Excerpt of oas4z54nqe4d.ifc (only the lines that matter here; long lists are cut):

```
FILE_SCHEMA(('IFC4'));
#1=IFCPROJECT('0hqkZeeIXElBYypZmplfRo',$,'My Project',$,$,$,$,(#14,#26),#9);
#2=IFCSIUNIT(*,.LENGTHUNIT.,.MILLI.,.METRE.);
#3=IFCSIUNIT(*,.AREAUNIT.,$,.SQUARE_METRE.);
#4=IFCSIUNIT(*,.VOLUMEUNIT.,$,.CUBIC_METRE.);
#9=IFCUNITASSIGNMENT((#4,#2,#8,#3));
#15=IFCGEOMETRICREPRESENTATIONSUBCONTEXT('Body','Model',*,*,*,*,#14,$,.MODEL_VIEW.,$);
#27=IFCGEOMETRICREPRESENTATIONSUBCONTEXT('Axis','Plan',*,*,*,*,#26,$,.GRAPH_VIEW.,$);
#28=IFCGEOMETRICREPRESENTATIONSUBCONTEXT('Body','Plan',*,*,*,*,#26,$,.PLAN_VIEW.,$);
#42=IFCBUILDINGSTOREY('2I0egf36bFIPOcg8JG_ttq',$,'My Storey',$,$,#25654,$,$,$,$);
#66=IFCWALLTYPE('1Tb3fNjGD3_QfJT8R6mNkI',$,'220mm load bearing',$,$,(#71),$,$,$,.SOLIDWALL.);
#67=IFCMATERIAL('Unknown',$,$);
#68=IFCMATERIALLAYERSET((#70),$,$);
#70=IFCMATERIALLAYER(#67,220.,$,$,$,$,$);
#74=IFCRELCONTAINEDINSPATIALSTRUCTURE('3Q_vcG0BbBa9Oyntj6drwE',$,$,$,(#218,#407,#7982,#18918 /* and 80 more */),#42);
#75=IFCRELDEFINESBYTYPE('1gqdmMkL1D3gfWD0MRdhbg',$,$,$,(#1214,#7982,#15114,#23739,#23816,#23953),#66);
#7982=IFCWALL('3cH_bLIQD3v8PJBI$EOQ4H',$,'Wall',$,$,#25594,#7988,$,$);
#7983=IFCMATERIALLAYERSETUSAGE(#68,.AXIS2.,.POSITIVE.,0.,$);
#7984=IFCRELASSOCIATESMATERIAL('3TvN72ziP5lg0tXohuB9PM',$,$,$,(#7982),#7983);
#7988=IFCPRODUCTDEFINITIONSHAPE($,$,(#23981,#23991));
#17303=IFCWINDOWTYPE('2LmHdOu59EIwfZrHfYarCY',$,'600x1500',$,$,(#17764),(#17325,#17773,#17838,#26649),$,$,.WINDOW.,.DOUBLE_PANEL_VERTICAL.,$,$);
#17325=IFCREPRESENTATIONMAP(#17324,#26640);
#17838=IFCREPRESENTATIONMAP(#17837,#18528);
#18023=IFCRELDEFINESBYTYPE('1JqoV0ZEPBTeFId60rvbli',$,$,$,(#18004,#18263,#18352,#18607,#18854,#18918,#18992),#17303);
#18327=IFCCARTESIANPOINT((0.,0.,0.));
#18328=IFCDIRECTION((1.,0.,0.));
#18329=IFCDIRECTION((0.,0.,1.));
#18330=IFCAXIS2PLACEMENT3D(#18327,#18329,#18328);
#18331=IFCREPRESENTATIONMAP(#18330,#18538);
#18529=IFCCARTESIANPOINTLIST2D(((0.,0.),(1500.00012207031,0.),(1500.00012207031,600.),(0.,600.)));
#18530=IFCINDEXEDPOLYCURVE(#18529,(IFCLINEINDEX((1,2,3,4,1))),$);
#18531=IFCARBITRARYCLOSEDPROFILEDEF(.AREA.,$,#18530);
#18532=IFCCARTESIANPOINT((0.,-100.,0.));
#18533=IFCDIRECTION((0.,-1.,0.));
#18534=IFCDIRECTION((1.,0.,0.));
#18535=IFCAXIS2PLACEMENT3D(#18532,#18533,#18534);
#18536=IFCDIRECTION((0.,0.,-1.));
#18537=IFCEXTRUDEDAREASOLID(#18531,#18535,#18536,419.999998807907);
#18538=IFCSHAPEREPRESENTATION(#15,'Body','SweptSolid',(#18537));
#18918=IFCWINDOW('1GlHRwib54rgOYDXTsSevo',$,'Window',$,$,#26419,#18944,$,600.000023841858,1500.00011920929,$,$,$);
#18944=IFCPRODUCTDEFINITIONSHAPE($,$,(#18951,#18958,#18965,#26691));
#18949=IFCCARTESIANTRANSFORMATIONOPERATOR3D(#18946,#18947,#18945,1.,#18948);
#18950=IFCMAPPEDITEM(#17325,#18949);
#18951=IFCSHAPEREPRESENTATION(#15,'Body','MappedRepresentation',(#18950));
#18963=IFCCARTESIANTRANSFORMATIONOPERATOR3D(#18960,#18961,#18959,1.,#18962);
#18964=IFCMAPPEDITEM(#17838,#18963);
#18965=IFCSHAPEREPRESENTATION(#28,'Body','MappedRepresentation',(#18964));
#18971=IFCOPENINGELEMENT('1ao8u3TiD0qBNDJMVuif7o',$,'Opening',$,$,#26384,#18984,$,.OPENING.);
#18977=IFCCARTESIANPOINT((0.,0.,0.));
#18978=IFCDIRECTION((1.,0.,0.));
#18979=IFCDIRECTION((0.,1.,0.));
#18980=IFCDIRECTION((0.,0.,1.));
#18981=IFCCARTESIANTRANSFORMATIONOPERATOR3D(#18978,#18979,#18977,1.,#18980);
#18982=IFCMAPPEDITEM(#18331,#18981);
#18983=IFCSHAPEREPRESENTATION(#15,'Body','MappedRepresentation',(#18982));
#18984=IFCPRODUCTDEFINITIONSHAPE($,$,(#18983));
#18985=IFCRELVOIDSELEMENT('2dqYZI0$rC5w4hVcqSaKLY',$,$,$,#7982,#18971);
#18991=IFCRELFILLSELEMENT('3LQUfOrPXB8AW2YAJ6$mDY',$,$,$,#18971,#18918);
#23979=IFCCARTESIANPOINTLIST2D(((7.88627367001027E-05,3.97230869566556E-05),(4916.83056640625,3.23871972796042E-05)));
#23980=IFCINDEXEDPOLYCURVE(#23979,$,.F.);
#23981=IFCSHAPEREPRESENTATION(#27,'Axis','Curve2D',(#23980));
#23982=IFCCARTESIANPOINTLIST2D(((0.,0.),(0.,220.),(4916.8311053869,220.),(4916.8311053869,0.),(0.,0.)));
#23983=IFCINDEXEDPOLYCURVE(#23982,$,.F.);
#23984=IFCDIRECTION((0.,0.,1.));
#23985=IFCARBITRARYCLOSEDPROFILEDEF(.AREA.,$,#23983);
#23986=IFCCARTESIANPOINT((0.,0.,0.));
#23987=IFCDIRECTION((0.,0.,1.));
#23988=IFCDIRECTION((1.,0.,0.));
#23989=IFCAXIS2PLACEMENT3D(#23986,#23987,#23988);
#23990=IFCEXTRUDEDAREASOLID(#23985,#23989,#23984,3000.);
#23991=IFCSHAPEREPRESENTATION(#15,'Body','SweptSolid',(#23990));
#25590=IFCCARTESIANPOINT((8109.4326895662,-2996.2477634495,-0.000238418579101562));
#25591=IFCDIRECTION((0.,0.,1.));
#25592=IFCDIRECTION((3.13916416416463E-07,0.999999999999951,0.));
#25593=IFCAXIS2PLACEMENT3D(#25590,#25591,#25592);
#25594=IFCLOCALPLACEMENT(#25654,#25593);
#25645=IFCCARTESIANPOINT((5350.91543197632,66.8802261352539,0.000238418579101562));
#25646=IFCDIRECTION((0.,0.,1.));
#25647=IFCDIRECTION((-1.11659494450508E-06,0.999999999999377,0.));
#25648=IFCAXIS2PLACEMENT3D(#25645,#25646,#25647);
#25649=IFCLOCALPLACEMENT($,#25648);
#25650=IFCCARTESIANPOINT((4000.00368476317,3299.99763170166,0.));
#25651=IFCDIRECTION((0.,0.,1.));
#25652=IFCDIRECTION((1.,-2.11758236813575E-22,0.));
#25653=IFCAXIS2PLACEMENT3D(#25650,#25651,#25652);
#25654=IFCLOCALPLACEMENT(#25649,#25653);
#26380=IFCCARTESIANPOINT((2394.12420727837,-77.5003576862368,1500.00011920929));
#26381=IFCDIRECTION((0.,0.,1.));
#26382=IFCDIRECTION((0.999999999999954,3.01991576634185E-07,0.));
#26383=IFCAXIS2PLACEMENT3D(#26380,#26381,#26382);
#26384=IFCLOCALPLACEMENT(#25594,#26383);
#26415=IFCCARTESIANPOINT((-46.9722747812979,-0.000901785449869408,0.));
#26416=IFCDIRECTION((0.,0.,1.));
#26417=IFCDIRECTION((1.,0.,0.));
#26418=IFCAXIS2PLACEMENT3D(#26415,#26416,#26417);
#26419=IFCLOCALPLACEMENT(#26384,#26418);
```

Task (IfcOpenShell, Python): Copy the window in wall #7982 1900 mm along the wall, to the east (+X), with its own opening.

```python
import ifcopenshell
import ifcopenshell.api.feature
import ifcopenshell.api.geometry
import ifcopenshell.api.root
import ifcopenshell.geom
import ifcopenshell.util.element
import ifcopenshell.util.placement
import ifcopenshell.util.shape
import ifcopenshell.util.unit

model = ifcopenshell.open("oas4z54nqe4d.ifc")
unit_scale = ifcopenshell.util.unit.calculate_unit_scale(model)
settings = ifcopenshell.geom.settings()


def volume(element):
    """Net volume in cubic metres, openings subtracted."""
    shape = ifcopenshell.geom.create_shape(settings, element)
    return ifcopenshell.util.shape.get_volume(shape.geometry)


window = model.by_id(18918)
opening = window.FillsVoids[0].RelatingOpeningElement
wall = opening.VoidsElements[0].RelatingBuildingElement
before = volume(wall)
shift = ifcopenshell.util.placement.get_local_placement(wall.ObjectPlacement)[:3, 0] * -1.9 / unit_scale

# copy_class copies the void relationship, type, container and properties, but no geometry.
new_opening = ifcopenshell.api.root.copy_class(model, product=opening)
new_opening.Representation = ifcopenshell.util.element.copy_deep(
    model, opening.Representation, exclude=["IfcGeometricRepresentationContext", "IfcRepresentationMap"]
)
new_window = ifcopenshell.api.root.copy_class(model, product=window)
new_window.Representation = ifcopenshell.util.element.copy_deep(
    model, window.Representation, exclude=["IfcGeometricRepresentationContext", "IfcRepresentationMap"]
)
ifcopenshell.api.feature.add_filling(model, opening=new_opening, element=new_window)

for old, new in ((opening, new_opening), (window, new_window)):
    matrix = ifcopenshell.util.placement.get_local_placement(old.ObjectPlacement)
    matrix[:3, 3] += shift
    ifcopenshell.api.geometry.edit_object_placement(model, product=new, matrix=matrix, is_si=False)

after = volume(wall)

print(f"wall volume {before:.3f} -> {after:.3f} m3")

model.write("oas4z54nqe4d_v2.ifc")
```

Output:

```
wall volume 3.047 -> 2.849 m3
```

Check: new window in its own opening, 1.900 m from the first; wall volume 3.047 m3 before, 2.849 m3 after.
